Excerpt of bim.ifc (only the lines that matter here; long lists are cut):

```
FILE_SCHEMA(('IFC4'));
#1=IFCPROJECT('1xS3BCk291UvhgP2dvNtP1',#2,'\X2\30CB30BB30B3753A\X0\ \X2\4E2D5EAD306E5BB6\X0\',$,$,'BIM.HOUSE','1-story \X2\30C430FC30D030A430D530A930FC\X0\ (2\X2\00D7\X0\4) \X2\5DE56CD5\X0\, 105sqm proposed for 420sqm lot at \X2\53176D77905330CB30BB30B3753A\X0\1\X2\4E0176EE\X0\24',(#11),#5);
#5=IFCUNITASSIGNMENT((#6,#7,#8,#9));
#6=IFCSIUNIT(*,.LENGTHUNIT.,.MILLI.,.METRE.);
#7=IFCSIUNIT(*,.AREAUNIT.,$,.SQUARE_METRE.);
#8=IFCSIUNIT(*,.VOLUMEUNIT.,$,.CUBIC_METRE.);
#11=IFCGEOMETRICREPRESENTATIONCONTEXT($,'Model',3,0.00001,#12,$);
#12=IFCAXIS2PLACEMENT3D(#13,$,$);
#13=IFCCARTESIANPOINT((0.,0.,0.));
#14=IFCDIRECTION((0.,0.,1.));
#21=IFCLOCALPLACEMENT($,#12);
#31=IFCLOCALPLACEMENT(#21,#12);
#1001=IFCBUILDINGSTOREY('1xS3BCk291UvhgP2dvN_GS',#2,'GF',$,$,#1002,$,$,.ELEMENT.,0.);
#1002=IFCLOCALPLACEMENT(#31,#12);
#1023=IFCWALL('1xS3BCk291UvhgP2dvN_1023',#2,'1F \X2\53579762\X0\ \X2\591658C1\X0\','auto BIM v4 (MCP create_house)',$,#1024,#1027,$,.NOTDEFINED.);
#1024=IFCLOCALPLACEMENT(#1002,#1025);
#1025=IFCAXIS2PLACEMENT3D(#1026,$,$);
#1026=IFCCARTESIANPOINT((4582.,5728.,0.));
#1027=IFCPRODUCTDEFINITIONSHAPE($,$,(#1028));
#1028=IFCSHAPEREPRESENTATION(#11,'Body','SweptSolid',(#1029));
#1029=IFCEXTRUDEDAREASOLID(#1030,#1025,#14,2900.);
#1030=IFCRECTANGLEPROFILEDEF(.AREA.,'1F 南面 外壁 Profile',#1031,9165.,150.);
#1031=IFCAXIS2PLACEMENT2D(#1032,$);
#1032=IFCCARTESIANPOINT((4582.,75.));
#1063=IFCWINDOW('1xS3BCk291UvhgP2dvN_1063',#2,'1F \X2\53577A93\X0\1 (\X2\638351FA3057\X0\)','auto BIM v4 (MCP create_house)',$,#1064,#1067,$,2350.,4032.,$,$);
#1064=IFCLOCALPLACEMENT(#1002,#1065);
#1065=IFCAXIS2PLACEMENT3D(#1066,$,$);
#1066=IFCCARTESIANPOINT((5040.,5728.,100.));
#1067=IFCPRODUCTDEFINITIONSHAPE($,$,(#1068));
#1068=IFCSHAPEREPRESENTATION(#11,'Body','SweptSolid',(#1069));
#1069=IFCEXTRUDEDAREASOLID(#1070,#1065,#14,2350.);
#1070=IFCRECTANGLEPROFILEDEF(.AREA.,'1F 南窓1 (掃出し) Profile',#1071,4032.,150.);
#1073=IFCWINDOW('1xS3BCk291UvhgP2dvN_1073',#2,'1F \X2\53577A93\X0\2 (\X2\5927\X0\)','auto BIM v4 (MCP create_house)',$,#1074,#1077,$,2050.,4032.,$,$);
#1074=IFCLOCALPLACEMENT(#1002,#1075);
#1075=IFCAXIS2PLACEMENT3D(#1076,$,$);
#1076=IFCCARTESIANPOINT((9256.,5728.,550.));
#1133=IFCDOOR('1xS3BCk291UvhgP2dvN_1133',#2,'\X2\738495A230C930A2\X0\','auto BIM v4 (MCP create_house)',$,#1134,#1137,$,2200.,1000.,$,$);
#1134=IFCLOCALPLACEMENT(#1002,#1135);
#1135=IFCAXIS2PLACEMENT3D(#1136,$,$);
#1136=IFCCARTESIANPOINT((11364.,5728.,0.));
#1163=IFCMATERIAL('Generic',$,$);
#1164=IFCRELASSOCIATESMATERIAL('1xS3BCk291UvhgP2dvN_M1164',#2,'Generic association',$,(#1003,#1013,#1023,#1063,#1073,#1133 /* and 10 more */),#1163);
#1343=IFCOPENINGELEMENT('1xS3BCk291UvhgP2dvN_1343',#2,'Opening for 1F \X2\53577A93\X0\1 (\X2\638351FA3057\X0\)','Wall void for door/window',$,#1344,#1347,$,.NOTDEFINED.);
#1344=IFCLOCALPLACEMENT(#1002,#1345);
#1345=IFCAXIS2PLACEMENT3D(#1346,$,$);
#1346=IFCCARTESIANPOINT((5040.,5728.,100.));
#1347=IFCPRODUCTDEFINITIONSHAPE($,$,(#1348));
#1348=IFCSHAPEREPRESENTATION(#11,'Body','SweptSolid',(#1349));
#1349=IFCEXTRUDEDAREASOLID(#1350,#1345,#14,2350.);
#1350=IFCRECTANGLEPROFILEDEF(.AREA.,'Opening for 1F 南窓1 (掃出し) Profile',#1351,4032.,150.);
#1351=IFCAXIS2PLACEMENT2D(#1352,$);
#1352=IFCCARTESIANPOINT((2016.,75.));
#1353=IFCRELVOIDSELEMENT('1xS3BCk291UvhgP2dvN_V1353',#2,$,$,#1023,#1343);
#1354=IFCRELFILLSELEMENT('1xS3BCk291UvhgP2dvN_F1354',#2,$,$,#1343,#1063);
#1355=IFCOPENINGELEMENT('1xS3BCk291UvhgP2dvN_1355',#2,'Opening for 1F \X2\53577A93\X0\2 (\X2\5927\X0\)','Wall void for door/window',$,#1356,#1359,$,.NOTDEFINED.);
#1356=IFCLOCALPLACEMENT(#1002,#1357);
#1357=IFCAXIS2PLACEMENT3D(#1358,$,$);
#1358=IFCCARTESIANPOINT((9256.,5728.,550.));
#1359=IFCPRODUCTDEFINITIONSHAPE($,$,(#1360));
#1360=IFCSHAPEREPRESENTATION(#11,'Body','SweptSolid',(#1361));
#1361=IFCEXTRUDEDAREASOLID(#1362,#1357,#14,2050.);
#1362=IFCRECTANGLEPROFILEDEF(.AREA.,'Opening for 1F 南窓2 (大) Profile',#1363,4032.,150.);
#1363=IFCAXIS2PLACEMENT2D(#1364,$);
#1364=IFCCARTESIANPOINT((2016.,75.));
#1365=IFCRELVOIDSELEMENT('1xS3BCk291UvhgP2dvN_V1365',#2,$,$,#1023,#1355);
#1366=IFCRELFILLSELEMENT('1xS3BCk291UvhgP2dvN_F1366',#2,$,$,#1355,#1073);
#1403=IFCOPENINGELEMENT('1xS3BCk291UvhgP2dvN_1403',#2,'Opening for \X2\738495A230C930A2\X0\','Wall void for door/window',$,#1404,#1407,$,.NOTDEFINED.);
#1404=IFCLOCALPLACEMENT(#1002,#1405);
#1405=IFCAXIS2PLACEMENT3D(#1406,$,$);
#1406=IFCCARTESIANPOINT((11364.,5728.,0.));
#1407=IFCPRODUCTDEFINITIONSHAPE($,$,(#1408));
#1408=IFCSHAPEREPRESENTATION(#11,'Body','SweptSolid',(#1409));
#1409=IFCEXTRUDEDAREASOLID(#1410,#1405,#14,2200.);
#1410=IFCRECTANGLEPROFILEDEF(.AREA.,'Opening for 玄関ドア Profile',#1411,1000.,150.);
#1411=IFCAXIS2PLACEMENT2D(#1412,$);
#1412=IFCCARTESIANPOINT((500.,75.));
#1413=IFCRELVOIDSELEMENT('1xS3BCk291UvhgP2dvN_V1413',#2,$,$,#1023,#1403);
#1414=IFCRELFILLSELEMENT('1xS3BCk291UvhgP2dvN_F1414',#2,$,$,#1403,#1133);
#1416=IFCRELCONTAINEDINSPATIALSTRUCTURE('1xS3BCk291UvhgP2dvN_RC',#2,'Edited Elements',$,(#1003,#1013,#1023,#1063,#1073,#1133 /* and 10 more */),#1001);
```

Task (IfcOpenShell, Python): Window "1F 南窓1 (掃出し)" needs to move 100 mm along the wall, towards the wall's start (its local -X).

```python
import ifcopenshell
import ifcopenshell.api.geometry
import ifcopenshell.util.placement
import ifcopenshell.util.unit

model = ifcopenshell.open("bim.ifc")
unit_scale = ifcopenshell.util.unit.calculate_unit_scale(model)

window = model.by_id(1063)
opening = window.FillsVoids[0].RelatingOpeningElement
wall = opening.VoidsElements[0].RelatingBuildingElement

wall_matrix = ifcopenshell.util.placement.get_local_placement(wall.ObjectPlacement)
shift = wall_matrix[:3, 0] * -0.1 / unit_scale
before = ifcopenshell.util.placement.get_local_placement(window.ObjectPlacement)[:3, 3].copy()

# The window is not placed relative to its opening, so move both.
for product in (opening, window):
    matrix = ifcopenshell.util.placement.get_local_placement(product.ObjectPlacement)
    matrix[:3, 3] += shift
    ifcopenshell.api.geometry.edit_object_placement(model, product=product, matrix=matrix, is_si=False)

after = ifcopenshell.util.placement.get_local_placement(window.ObjectPlacement)[:3, 3]
print("window moved by", (after - before).round(3) + 0.0)

model.write("bim_v2.ifc")
```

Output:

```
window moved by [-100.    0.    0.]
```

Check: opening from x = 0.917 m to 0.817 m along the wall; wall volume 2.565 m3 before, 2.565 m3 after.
